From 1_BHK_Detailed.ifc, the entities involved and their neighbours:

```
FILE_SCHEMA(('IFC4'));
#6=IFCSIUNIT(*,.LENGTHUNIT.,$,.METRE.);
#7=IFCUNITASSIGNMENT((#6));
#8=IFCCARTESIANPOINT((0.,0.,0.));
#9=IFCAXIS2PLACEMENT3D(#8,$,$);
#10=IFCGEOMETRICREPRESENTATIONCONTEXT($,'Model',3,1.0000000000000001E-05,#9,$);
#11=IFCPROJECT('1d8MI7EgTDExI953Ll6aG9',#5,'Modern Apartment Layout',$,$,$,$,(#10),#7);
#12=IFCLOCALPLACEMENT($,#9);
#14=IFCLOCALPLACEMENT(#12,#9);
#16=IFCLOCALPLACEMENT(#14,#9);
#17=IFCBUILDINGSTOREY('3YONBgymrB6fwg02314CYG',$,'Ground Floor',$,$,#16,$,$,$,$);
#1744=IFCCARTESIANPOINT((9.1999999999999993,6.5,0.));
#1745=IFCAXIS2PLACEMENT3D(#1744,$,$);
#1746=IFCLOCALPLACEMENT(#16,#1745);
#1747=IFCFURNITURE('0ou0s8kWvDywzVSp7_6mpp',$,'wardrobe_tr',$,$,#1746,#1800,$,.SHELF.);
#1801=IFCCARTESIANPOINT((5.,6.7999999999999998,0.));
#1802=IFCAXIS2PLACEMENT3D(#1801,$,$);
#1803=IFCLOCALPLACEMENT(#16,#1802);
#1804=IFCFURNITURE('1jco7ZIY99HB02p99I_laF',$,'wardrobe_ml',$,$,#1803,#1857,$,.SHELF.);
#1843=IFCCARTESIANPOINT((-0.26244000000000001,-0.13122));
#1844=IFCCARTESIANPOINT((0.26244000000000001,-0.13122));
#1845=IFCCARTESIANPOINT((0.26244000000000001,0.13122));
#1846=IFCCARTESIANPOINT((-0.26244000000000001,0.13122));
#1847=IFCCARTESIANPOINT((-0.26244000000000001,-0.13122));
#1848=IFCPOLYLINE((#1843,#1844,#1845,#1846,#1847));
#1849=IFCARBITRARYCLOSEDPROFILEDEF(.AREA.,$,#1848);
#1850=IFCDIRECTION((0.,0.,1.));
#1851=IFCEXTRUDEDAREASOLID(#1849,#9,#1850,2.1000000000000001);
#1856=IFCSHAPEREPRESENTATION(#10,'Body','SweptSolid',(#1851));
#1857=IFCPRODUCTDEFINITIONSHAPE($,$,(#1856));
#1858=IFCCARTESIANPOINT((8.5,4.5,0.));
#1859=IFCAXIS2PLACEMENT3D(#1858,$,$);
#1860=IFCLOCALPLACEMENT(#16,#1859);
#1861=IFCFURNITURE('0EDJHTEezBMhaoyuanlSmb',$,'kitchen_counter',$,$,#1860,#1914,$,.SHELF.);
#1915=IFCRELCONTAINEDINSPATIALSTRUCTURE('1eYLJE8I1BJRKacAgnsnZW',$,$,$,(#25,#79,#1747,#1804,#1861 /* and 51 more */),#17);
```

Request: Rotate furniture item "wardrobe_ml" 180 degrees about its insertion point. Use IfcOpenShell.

```python
import ifcopenshell
import ifcopenshell.api.geometry
import ifcopenshell.util.placement

model = ifcopenshell.open("1_BHK_Detailed.ifc")

item = model.by_guid("1jco7ZIY99HB02p99I_laF")
matrix = ifcopenshell.util.placement.get_local_placement(item.ObjectPlacement)
matrix = matrix @ ifcopenshell.util.placement.rotation(180, "Z")
ifcopenshell.api.geometry.edit_object_placement(model, product=item, matrix=matrix, is_si=False)

print(ifcopenshell.util.placement.get_local_placement(item.ObjectPlacement).round(3) + 0.0)

model.write("1_BHK_Detailed_rev.ifc")
```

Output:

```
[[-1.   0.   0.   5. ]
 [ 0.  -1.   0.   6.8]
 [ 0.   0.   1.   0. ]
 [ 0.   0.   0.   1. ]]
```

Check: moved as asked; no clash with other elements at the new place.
